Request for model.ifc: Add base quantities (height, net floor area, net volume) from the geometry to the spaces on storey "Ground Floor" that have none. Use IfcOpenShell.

First a look at what the model holds.

```python
import ifcopenshell
import ifcopenshell.util.element
import ifcopenshell.util.unit

model = ifcopenshell.open("model.ifc")
print(model.schema)
for unit_type in ("LENGTHUNIT", "AREAUNIT", "VOLUMEUNIT"):
    print(unit_type, ifcopenshell.util.unit.calculate_unit_scale(model, unit_type))
storey = next(s for s in model.by_type("IfcBuildingStorey") if s.Name == "Ground Floor")
spaces = [e for e in ifcopenshell.util.element.get_decomposition(storey) if e.is_a("IfcSpace")]
for e in sorted(spaces, key=lambda e: e.id()):
    print(e.id(), e.is_a(), e.Name, list(ifcopenshell.util.element.get_psets(e, qtos_only=True)), sep=" | ")
```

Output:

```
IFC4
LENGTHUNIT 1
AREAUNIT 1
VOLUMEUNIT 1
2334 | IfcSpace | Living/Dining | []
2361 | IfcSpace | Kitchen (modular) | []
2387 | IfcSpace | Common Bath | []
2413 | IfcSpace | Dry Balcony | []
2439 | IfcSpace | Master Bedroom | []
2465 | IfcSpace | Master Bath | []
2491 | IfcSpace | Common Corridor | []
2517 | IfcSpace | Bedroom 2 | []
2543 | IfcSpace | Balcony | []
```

```python
import ifcopenshell
import ifcopenshell.api.pset
import ifcopenshell.geom
import ifcopenshell.util.element
import ifcopenshell.util.shape
import ifcopenshell.util.unit

model = ifcopenshell.open("model.ifc")
unit_scale = ifcopenshell.util.unit.calculate_unit_scale(model)
area_scale = ifcopenshell.util.unit.calculate_unit_scale(model, "AREAUNIT")
volume_scale = ifcopenshell.util.unit.calculate_unit_scale(model, "VOLUMEUNIT")
settings = ifcopenshell.geom.settings()

storey = next(s for s in model.by_type("IfcBuildingStorey") if s.Name == "Ground Floor")
spaces = [e for e in ifcopenshell.util.element.get_decomposition(storey) if e.is_a("IfcSpace")]

for e in sorted(spaces, key=lambda e: e.id()):
    if ifcopenshell.util.element.get_psets(e, qtos_only=True, should_inherit=False):
        continue
    # Geometry comes back in metres, in the element's own axes.
    shape = ifcopenshell.geom.create_shape(settings, e)
    values = {
        "Height": ifcopenshell.util.shape.get_z(shape.geometry) / unit_scale,
        "NetFloorArea": ifcopenshell.util.shape.get_footprint_area(shape.geometry) / area_scale,
        "NetVolume": ifcopenshell.util.shape.get_volume(shape.geometry) / volume_scale,
    }
    qto = ifcopenshell.api.pset.add_qto(model, product=e, name="Qto_SpaceBaseQuantities")
    ifcopenshell.api.pset.edit_qto(model, qto=qto, properties=values)
    print(e.id(), {k: round(v, 3) for k, v in values.items()})

model.write("model_rev.ifc")
```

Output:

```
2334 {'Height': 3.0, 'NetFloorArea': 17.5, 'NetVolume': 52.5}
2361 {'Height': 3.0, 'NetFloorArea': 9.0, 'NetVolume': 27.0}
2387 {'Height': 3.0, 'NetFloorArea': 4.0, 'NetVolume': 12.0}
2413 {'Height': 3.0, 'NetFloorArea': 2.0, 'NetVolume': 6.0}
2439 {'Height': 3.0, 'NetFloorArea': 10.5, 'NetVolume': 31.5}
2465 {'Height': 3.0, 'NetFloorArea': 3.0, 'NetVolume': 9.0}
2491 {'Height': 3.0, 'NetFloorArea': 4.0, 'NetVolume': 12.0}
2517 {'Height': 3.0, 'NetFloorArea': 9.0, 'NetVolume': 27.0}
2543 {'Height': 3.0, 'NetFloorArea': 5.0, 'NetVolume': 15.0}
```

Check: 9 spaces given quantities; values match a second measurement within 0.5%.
